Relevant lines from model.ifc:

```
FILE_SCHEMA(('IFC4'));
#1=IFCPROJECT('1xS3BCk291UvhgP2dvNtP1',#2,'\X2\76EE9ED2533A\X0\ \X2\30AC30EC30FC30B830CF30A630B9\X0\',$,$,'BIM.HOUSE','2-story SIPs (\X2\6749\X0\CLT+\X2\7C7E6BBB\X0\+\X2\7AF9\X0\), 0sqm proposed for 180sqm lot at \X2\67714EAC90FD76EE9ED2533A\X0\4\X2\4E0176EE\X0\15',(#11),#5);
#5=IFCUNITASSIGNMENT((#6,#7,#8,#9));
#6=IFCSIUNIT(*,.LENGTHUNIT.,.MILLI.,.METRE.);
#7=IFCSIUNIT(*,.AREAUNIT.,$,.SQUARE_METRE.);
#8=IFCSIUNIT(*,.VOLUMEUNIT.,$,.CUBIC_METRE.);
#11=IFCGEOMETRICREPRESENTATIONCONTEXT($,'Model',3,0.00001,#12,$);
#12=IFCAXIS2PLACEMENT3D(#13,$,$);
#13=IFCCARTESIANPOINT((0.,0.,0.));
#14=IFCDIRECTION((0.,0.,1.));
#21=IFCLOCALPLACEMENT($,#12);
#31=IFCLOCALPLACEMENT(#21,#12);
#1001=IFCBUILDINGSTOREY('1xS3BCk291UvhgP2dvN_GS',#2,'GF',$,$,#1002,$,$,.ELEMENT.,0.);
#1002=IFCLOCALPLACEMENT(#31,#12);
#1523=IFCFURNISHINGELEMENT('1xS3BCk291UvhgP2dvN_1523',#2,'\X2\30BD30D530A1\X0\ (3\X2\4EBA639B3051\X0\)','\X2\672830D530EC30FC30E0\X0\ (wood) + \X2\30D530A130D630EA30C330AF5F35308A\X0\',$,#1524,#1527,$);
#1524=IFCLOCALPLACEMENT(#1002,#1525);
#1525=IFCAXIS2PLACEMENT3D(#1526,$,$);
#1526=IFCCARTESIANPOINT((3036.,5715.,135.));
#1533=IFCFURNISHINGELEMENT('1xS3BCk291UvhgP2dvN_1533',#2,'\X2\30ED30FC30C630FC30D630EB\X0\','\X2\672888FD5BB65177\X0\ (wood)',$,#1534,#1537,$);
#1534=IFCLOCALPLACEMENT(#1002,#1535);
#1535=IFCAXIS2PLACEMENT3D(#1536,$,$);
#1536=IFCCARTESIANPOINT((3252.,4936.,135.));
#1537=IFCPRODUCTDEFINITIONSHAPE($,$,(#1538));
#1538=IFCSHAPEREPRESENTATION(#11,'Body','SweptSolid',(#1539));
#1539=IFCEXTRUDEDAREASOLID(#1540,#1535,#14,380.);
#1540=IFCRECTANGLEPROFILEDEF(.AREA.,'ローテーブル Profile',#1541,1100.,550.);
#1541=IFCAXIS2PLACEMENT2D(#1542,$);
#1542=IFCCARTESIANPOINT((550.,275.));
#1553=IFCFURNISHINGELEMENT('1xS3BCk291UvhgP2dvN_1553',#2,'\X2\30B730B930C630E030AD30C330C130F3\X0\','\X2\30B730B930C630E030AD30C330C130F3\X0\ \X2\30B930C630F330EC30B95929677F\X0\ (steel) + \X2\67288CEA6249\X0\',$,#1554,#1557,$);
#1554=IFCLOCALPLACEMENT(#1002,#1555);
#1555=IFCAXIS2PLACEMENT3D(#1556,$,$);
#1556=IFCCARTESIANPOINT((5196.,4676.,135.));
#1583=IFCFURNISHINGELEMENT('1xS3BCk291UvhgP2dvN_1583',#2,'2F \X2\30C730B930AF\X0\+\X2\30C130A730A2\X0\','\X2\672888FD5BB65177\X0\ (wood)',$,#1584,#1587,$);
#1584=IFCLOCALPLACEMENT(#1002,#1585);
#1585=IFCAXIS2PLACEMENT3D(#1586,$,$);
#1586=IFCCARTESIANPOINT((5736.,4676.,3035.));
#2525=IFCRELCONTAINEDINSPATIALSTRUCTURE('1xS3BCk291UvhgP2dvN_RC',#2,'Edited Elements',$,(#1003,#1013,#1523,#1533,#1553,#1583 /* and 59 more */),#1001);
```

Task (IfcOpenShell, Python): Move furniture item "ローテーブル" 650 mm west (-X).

```python
import ifcopenshell
import ifcopenshell.api.geometry
import ifcopenshell.util.placement

model = ifcopenshell.open("model.ifc")

item = model.by_guid("1xS3BCk291UvhgP2dvN_1533")
matrix = ifcopenshell.util.placement.get_local_placement(item.ObjectPlacement)
matrix[0, 3] -= 650.0
ifcopenshell.api.geometry.edit_object_placement(model, product=item, matrix=matrix, is_si=False)

print(ifcopenshell.util.placement.get_local_placement(item.ObjectPlacement).round(3) + 0.0)

model.write("model_rev.ifc")
```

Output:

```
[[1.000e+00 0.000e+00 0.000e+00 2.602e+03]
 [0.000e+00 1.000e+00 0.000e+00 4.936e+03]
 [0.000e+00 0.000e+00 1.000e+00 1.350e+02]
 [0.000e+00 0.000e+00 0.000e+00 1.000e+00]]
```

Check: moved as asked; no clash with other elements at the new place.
